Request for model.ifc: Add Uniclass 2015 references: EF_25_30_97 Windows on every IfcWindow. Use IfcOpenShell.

First a look at what the model holds.

```python
import ifcopenshell

model = ifcopenshell.open("model.ifc")
print(model.schema)
print("classifications:", [c.Name for c in model.by_type("IfcClassification")])
for ifc_class in ("IfcDoor", "IfcRoof", "IfcStair", "IfcWall", "IfcWindow"):
    print(ifc_class, len(model.by_type(ifc_class)))
```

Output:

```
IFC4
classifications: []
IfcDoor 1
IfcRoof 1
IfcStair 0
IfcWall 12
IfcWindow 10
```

```python
import ifcopenshell
import ifcopenshell.api.classification

model = ifcopenshell.open("model.ifc")

system = ifcopenshell.api.classification.add_classification(model, classification="Uniclass 2015")

codes = {
    "IfcWindow": ("EF_25_30_97", "Windows"),
}
for ifc_class, (code, name) in codes.items():
    products = model.by_type(ifc_class)
    ifcopenshell.api.classification.add_reference(
        model, products=products, classification=system, identification=code, name=name
    )
    print(code, len(products))

model.write("model_rev.ifc")
```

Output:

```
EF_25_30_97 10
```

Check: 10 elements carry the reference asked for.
